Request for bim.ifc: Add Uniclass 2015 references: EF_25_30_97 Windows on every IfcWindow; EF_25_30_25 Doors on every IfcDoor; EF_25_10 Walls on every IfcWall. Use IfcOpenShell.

First a look at what the model holds.

```python
import ifcopenshell

model = ifcopenshell.open("bim.ifc")
print(model.schema)
print("classifications:", [c.Name for c in model.by_type("IfcClassification")])
for ifc_class in ("IfcDoor", "IfcRoof", "IfcStair", "IfcWall", "IfcWindow"):
    print(ifc_class, len(model.by_type(ifc_class)))
```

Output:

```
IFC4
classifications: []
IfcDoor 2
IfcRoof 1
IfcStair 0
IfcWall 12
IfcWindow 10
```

```python
import ifcopenshell
import ifcopenshell.api.classification

model = ifcopenshell.open("bim.ifc")

system = ifcopenshell.api.classification.add_classification(model, classification="Uniclass 2015")

codes = {
    "IfcWindow": ("EF_25_30_97", "Windows"),
    "IfcDoor": ("EF_25_30_25", "Doors"),
    "IfcWall": ("EF_25_10", "Walls"),
}
for ifc_class, (code, name) in codes.items():
    products = model.by_type(ifc_class)
    ifcopenshell.api.classification.add_reference(
        model, products=products, classification=system, identification=code, name=name
    )
    print(code, len(products))

model.write("bim_edited.ifc")
```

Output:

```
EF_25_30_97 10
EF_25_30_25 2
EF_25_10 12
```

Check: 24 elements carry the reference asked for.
